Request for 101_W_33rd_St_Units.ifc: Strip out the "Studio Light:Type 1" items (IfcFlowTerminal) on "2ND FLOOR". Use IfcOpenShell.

First a look at what the model holds.

```python
import ifcopenshell
import ifcopenshell.util.element

model = ifcopenshell.open("101_W_33rd_St_Units.ifc")
print(model.schema)
storey = next(s for s in model.by_type("IfcBuildingStorey") if s.Name == "2ND FLOOR")
terminals = [e for e in ifcopenshell.util.element.get_decomposition(storey) if e.is_a("IfcFlowTerminal")]
seen = {}
for e in terminals:
    element_type = ifcopenshell.util.element.get_type(e)
    name = element_type.Name if element_type not in (None, e) else None
    seen[name] = seen.get(name, 0) + 1
for name, count in sorted(seen.items(), key=str):
    print(count, "x", name)
```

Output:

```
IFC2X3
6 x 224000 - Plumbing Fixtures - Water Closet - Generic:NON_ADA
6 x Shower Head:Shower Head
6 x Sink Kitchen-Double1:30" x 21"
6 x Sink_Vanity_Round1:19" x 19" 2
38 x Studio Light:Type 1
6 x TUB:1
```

```python
import ifcopenshell
import ifcopenshell.api.root
import ifcopenshell.util.element

model = ifcopenshell.open("101_W_33rd_St_Units.ifc")

storey = next(s for s in model.by_type("IfcBuildingStorey") if s.Name == "2ND FLOOR")
terminals = [e for e in ifcopenshell.util.element.get_decomposition(storey) if e.is_a("IfcFlowTerminal")]
targets = [e for e in terminals if (t := ifcopenshell.util.element.get_type(e)) not in (None, e) and t.Name == "Studio Light:Type 1"]

for e in targets:
    ifcopenshell.api.root.remove_product(model, product=e)
print(len(targets), "removed")

model.write("101_W_33rd_St_Units_updated.ifc")
```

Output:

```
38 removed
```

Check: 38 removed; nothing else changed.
